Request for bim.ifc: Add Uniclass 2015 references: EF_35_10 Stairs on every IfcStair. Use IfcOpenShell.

First a look at what the model holds.

```python
import ifcopenshell

model = ifcopenshell.open("bim.ifc")
print(model.schema)
print("classifications:", [c.Name for c in model.by_type("IfcClassification")])
for ifc_class in ("IfcDoor", "IfcRoof", "IfcStair", "IfcWall", "IfcWindow"):
    print(ifc_class, len(model.by_type(ifc_class)))
```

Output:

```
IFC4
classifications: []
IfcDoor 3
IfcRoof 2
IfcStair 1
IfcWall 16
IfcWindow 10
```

```python
import ifcopenshell
import ifcopenshell.api.classification

model = ifcopenshell.open("bim.ifc")

system = ifcopenshell.api.classification.add_classification(model, classification="Uniclass 2015")

codes = {
    "IfcStair": ("EF_35_10", "Stairs"),
}
for ifc_class, (code, name) in codes.items():
    products = model.by_type(ifc_class)
    ifcopenshell.api.classification.add_reference(
        model, products=products, classification=system, identification=code, name=name
    )
    print(code, len(products))

model.write("bim_rev.ifc")
```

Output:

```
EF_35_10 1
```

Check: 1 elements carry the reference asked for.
